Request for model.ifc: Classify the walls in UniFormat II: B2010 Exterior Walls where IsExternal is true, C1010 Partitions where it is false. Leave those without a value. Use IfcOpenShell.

First a look at what the model holds.

```python
import ifcopenshell
import ifcopenshell.util.element

model = ifcopenshell.open("model.ifc")
print(model.schema)
print("classifications:", [c.Name for c in model.by_type("IfcClassification")])
values = [ifcopenshell.util.element.get_pset(e, "Pset_WallCommon", "IsExternal") for e in model.by_type("IfcWall")]
for value in (True, False, None):
    print("IsExternal", value, values.count(value))
```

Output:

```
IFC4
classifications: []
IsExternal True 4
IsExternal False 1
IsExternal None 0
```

```python
import ifcopenshell
import ifcopenshell.api.classification
import ifcopenshell.util.element

model = ifcopenshell.open("model.ifc")

system = ifcopenshell.api.classification.add_classification(model, classification="UniFormat II")

walls = model.by_type("IfcWall")
external = {e: ifcopenshell.util.element.get_pset(e, "Pset_WallCommon", "IsExternal") for e in walls}
for flag, code, name in ((True, "B2010", "Exterior Walls"), (False, "C1010", "Partitions")):
    products = [e for e in walls if external[e] is flag]
    ifcopenshell.api.classification.add_reference(
        model, products=products, classification=system, identification=code, name=name
    )
    print(code, len(products))

model.write("model_edited.ifc")
```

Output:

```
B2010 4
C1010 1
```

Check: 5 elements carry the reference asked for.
